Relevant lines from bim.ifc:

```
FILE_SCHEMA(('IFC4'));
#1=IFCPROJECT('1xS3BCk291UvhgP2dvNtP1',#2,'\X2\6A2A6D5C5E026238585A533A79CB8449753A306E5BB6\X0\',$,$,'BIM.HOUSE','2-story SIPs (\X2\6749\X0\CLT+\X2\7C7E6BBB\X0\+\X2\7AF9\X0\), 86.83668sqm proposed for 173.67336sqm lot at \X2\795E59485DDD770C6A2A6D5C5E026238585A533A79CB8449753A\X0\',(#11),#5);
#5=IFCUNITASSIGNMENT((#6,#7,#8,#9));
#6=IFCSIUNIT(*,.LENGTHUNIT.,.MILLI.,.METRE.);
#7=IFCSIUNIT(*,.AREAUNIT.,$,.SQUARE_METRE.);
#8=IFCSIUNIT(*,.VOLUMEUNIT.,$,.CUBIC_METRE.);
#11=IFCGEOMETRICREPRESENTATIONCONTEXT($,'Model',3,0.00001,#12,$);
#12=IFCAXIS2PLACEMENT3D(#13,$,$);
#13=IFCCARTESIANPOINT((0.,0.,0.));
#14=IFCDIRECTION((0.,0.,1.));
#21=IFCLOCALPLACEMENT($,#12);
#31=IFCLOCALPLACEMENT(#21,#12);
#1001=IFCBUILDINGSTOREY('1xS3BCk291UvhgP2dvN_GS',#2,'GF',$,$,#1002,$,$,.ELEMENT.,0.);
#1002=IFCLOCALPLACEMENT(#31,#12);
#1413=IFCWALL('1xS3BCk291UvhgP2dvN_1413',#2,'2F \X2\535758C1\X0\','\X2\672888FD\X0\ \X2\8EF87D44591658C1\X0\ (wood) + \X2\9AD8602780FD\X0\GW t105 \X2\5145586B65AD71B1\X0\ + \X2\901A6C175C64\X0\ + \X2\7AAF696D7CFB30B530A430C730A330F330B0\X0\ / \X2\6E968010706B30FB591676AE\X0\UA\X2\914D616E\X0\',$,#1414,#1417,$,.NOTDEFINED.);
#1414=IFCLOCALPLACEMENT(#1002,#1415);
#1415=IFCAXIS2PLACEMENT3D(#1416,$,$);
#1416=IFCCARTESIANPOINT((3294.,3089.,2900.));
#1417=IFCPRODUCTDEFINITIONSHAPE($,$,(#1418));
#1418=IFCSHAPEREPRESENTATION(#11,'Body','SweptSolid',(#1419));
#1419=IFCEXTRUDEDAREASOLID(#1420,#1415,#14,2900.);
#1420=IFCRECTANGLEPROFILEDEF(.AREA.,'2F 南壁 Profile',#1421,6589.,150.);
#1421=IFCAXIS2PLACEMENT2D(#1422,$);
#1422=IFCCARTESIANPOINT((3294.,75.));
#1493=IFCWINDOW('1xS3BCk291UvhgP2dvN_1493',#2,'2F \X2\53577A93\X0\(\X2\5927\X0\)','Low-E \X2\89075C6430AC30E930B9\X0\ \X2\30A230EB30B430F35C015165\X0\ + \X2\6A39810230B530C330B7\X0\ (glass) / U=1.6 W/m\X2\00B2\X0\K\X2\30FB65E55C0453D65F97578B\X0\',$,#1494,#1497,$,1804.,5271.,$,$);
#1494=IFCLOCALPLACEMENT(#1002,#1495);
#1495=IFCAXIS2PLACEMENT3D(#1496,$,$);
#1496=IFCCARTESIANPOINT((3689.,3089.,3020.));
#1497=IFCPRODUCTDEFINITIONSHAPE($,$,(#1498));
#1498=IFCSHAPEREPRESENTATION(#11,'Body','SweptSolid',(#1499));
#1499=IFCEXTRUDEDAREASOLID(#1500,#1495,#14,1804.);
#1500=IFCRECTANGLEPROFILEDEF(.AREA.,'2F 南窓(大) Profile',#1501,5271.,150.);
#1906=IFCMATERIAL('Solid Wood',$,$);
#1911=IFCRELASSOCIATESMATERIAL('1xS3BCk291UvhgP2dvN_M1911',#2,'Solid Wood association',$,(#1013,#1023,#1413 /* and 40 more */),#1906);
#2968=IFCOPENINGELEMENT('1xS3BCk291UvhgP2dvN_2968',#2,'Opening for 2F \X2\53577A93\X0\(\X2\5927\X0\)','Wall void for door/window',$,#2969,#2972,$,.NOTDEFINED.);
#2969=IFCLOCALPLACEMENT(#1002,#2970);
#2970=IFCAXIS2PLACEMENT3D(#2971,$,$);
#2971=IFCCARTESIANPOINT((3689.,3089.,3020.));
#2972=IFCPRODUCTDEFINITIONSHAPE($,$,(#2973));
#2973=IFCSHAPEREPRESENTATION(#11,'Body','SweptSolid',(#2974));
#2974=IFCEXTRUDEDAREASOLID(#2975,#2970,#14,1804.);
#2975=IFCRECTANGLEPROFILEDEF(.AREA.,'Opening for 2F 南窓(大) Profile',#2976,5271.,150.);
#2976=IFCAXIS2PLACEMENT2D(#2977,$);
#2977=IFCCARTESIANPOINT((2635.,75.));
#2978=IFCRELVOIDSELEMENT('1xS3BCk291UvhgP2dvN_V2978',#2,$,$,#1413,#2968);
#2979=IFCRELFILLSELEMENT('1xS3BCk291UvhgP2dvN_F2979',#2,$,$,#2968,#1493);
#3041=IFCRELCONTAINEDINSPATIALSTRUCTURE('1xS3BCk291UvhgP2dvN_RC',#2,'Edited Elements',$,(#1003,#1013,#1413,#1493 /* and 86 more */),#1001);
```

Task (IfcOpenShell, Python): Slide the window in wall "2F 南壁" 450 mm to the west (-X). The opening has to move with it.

```python
import ifcopenshell
import ifcopenshell.api.geometry
import ifcopenshell.util.placement
import ifcopenshell.util.unit

model = ifcopenshell.open("bim.ifc")
unit_scale = ifcopenshell.util.unit.calculate_unit_scale(model)

window = model.by_guid("1xS3BCk291UvhgP2dvN_1493")
opening = window.FillsVoids[0].RelatingOpeningElement
wall = opening.VoidsElements[0].RelatingBuildingElement

wall_matrix = ifcopenshell.util.placement.get_local_placement(wall.ObjectPlacement)
shift = wall_matrix[:3, 0] * -0.45 / unit_scale
before = ifcopenshell.util.placement.get_local_placement(window.ObjectPlacement)[:3, 3].copy()

# The window is not placed relative to its opening, so move both.
for product in (opening, window):
    matrix = ifcopenshell.util.placement.get_local_placement(product.ObjectPlacement)
    matrix[:3, 3] += shift
    ifcopenshell.api.geometry.edit_object_placement(model, product=product, matrix=matrix, is_si=False)

after = ifcopenshell.util.placement.get_local_placement(window.ObjectPlacement)[:3, 3]
print("window moved by", (after - before).round(3) + 0.0)

model.write("bim_updated.ifc")
```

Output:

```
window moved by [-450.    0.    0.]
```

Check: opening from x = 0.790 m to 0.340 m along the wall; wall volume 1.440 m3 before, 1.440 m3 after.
